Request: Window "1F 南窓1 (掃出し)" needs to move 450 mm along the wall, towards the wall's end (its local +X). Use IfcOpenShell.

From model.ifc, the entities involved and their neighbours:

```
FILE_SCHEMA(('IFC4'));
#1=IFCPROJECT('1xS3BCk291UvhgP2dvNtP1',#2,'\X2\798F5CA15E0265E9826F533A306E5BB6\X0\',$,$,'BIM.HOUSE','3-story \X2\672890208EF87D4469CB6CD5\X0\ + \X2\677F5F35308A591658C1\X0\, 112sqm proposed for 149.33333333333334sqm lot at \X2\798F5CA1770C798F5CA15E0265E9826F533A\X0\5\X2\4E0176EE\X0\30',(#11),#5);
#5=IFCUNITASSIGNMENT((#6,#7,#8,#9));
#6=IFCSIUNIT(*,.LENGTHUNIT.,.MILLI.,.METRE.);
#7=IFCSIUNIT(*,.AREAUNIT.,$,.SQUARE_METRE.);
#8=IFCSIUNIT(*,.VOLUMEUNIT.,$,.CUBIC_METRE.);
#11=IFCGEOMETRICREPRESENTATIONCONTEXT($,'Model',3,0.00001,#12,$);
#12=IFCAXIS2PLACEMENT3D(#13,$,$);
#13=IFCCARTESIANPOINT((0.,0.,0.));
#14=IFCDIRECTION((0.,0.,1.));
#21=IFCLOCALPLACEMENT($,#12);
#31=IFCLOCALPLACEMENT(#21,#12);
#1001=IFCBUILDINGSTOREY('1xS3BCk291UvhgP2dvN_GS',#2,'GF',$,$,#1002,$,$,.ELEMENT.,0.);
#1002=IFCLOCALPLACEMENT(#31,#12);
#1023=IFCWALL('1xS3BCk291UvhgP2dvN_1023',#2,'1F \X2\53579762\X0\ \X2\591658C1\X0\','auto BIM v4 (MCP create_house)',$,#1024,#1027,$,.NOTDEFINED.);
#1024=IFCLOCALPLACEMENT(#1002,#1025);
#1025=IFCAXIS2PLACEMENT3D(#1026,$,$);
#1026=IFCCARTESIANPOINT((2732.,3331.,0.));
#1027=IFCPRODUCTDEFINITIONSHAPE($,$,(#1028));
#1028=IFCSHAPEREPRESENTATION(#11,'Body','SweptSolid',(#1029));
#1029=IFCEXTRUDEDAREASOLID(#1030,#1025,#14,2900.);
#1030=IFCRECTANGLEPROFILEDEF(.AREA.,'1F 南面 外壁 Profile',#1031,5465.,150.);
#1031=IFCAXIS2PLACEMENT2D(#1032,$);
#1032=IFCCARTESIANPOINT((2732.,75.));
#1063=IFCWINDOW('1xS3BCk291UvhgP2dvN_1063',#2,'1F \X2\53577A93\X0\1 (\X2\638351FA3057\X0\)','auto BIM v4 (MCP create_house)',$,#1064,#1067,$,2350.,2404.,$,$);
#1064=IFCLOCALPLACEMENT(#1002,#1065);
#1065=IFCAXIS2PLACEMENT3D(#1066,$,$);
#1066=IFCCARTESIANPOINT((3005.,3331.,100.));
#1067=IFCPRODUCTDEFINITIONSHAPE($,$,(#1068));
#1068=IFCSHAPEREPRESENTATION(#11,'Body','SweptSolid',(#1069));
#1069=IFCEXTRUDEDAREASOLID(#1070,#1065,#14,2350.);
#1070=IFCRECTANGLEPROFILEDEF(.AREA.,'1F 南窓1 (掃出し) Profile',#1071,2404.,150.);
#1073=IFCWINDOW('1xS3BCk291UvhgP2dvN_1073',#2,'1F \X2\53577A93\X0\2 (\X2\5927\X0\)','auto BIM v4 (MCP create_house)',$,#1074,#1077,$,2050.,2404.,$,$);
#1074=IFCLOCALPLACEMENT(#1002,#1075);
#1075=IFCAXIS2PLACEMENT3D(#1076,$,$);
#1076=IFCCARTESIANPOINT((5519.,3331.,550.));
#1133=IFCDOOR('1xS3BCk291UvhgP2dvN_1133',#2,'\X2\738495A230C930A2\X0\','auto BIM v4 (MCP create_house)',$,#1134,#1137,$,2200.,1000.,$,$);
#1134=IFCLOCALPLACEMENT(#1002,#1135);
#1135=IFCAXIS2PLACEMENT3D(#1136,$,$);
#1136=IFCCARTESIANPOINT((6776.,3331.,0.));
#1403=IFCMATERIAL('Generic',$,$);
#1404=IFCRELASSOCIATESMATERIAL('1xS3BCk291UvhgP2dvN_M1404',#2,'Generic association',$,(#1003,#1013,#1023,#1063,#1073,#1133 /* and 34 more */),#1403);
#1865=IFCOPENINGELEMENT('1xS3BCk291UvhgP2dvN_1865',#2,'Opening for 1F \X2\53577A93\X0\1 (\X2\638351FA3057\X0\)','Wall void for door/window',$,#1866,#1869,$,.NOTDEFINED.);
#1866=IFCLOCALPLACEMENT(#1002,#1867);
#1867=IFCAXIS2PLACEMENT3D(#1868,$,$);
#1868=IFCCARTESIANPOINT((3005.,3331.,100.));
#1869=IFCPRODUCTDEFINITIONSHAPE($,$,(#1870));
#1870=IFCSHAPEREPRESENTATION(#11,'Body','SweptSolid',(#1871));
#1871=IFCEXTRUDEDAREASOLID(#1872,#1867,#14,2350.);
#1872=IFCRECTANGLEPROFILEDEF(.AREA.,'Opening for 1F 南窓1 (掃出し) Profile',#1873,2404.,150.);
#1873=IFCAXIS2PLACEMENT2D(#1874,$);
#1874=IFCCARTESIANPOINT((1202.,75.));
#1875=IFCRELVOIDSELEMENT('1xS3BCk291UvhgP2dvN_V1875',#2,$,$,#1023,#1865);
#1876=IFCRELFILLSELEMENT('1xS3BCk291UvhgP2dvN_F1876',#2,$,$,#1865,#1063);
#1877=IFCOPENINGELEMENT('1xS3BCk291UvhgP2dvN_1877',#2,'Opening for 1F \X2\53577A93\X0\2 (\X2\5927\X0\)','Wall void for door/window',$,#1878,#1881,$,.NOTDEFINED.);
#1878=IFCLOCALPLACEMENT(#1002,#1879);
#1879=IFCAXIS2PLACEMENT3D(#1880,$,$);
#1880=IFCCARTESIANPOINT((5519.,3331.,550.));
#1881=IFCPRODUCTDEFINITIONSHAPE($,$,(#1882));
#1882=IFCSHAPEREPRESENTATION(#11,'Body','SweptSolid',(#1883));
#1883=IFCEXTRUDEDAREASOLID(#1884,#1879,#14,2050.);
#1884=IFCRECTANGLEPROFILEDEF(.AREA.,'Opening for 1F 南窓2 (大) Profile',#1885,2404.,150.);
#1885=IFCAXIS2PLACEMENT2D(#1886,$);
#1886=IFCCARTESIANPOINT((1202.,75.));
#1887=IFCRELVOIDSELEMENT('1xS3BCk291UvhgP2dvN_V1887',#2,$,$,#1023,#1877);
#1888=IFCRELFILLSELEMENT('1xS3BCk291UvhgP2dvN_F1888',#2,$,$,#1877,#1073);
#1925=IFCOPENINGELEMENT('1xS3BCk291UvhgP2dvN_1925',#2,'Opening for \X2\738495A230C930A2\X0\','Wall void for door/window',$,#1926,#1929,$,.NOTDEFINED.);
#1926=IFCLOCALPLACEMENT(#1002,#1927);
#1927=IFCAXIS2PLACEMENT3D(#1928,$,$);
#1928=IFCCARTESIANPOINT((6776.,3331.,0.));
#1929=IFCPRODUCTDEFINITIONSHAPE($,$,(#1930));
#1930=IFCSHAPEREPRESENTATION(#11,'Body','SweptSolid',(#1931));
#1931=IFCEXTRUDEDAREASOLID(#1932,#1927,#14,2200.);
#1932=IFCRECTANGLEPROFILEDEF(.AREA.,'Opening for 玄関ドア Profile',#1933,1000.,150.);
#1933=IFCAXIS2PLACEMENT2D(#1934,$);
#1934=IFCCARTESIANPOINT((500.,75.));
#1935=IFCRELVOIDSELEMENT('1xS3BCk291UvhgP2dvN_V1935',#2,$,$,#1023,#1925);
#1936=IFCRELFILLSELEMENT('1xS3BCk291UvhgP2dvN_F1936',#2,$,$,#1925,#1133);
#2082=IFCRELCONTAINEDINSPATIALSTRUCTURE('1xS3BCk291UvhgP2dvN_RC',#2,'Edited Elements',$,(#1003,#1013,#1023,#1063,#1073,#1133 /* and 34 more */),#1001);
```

```python
import ifcopenshell
import ifcopenshell.api.geometry
import ifcopenshell.util.placement

model = ifcopenshell.open("model.ifc")

window = model.by_guid("1xS3BCk291UvhgP2dvN_1063")
opening = window.FillsVoids[0].RelatingOpeningElement
wall = opening.VoidsElements[0].RelatingBuildingElement

wall_matrix = ifcopenshell.util.placement.get_local_placement(wall.ObjectPlacement)
shift = wall_matrix[:3, 0] * 450.0
before = ifcopenshell.util.placement.get_local_placement(window.ObjectPlacement)[:3, 3].copy()

# The window is not placed relative to its opening, so move both.
for product in (opening, window):
    matrix = ifcopenshell.util.placement.get_local_placement(product.ObjectPlacement)
    matrix[:3, 3] += shift
    ifcopenshell.api.geometry.edit_object_placement(model, product=product, matrix=matrix, is_si=False)

after = ifcopenshell.util.placement.get_local_placement(window.ObjectPlacement)[:3, 3]
print("window moved by", (after - before).round(3) + 0.0)

model.write("model_v2.ifc")
```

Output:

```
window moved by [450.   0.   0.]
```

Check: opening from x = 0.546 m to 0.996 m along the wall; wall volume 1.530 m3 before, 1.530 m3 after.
